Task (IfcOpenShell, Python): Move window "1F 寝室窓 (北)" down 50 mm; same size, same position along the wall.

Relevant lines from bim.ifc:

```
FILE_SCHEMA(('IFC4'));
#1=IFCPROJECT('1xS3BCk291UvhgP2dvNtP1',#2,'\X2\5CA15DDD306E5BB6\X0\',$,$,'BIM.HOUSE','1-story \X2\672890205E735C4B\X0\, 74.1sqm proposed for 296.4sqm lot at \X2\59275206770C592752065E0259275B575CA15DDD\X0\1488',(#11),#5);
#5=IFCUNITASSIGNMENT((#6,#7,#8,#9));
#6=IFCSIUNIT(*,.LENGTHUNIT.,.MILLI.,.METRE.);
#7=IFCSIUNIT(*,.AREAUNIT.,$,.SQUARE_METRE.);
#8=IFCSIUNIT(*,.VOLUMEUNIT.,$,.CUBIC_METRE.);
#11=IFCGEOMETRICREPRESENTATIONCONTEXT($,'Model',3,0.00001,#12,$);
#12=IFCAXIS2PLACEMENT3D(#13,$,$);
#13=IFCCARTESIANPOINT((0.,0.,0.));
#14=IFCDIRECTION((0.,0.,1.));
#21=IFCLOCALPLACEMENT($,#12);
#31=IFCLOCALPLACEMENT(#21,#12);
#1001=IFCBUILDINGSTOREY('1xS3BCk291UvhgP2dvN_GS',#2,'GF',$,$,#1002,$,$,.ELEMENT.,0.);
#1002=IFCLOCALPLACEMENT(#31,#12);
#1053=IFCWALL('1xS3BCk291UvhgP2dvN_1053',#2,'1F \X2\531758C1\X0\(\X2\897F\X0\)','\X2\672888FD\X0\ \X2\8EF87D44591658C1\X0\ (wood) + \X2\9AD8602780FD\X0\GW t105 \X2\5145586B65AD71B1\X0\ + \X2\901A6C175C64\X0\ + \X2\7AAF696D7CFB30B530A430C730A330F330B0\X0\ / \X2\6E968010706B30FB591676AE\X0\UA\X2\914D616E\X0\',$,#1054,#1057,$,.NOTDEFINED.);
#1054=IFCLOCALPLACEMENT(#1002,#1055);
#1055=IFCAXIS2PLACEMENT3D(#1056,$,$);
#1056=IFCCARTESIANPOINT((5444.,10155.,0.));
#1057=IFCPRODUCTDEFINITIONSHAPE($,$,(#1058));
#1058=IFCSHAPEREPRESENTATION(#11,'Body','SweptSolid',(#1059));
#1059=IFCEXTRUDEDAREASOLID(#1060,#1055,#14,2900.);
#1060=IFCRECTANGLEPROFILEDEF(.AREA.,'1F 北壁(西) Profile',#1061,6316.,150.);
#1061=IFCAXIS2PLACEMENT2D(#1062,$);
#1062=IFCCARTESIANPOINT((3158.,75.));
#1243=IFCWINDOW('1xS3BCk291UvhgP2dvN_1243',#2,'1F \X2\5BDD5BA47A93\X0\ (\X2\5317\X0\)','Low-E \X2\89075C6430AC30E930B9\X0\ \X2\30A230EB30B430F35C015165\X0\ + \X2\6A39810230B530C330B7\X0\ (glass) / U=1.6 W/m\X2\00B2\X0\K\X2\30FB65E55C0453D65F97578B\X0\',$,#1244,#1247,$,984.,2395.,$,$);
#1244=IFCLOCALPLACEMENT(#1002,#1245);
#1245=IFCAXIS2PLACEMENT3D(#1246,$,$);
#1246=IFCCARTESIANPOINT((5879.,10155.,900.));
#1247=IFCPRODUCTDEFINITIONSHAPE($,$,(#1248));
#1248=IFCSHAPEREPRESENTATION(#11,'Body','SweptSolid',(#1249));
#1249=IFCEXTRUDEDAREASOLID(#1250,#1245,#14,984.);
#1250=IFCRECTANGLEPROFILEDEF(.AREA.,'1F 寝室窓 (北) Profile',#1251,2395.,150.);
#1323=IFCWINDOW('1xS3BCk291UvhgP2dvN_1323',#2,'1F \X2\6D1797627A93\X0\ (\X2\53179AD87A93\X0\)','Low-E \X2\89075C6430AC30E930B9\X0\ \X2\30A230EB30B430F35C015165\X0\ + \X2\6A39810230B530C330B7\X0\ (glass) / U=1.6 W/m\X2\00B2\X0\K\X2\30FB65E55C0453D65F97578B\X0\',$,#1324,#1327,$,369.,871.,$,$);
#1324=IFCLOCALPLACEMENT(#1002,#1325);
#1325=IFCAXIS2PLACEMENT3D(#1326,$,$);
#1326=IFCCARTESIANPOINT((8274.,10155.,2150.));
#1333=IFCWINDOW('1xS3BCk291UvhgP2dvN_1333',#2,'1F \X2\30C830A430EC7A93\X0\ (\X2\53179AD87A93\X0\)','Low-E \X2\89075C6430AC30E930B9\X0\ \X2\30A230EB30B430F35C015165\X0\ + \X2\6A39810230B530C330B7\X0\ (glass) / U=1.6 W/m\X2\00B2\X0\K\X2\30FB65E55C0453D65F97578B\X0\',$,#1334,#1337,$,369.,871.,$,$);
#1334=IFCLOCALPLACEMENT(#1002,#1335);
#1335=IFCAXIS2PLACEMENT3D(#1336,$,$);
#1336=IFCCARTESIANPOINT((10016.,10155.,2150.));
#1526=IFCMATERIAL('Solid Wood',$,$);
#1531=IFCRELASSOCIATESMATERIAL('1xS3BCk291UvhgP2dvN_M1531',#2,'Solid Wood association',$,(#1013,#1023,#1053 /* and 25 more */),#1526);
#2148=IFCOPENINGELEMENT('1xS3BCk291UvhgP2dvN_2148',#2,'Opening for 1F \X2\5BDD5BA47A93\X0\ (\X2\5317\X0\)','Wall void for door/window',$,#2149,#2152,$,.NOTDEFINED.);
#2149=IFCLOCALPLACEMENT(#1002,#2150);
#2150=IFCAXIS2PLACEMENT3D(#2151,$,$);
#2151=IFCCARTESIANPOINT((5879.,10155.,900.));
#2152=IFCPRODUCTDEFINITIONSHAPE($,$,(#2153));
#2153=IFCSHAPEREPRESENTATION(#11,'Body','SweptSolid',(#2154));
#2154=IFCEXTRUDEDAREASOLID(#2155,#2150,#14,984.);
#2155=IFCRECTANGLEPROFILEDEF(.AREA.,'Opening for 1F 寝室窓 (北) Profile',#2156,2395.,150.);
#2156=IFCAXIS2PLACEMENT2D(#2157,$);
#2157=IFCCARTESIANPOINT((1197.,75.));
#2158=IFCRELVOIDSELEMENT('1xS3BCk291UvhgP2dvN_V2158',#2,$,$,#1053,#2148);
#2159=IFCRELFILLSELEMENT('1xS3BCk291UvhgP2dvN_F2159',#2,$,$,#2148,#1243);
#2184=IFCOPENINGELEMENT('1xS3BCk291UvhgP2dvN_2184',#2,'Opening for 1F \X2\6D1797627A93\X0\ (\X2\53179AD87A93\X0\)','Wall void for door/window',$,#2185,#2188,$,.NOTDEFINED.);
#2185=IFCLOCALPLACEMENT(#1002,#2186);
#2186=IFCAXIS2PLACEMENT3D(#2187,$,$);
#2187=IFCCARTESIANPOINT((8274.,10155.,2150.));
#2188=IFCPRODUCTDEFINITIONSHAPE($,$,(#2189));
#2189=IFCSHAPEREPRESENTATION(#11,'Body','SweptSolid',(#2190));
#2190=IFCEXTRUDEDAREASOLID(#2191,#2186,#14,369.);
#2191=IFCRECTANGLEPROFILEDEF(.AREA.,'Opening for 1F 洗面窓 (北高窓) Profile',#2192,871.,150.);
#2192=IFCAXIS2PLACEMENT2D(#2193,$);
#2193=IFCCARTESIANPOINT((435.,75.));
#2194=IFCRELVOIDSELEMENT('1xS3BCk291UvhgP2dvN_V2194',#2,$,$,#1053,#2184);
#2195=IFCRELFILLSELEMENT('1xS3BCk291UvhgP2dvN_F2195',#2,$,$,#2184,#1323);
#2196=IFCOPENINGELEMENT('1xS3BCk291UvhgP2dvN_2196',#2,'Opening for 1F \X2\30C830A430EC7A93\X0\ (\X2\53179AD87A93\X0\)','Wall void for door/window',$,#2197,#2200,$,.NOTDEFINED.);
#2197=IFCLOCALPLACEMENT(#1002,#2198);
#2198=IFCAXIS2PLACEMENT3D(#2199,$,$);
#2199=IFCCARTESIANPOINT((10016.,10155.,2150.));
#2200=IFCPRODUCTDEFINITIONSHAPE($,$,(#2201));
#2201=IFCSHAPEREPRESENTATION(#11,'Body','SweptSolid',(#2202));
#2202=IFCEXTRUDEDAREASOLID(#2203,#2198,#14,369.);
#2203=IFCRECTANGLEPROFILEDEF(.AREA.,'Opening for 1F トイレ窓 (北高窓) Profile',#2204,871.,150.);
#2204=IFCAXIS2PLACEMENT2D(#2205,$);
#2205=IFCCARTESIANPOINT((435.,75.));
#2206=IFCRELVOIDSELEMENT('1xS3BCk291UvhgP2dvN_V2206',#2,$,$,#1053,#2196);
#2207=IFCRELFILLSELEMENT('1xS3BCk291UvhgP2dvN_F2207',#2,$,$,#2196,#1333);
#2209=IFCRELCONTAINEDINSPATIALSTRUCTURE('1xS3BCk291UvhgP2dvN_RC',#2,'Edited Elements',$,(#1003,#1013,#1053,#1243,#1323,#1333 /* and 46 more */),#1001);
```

```python
import numpy as np
import ifcopenshell
import ifcopenshell.api.geometry
import ifcopenshell.util.placement
import ifcopenshell.util.unit

model = ifcopenshell.open("bim.ifc")
unit_scale = ifcopenshell.util.unit.calculate_unit_scale(model)

window = model.by_guid("1xS3BCk291UvhgP2dvN_1243")
opening = window.FillsVoids[0].RelatingOpeningElement
dz = -0.05 / unit_scale

shift = np.array([0.0, 0.0, dz])
# The window is not placed relative to its opening, so move both.
for product in (opening, window):
    matrix = ifcopenshell.util.placement.get_local_placement(product.ObjectPlacement)
    matrix[:3, 3] += shift
    ifcopenshell.api.geometry.edit_object_placement(model, product=product, matrix=matrix, is_si=False)

print(f"moved by {dz * unit_scale:+.3f} m")

model.write("bim_edited.ifc")
```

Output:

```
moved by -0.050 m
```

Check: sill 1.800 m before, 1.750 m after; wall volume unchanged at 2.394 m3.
